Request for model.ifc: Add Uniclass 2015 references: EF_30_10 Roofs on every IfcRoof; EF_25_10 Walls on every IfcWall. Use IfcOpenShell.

First a look at what the model holds.

```python
import ifcopenshell

model = ifcopenshell.open("model.ifc")
print(model.schema)
print("classifications:", [c.Name for c in model.by_type("IfcClassification")])
for ifc_class in ("IfcDoor", "IfcRoof", "IfcStair", "IfcWall", "IfcWindow"):
    print(ifc_class, len(model.by_type(ifc_class)))
```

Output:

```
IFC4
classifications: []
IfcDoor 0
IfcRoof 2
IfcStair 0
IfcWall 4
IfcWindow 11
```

```python
import ifcopenshell
import ifcopenshell.api.classification

model = ifcopenshell.open("model.ifc")

system = ifcopenshell.api.classification.add_classification(model, classification="Uniclass 2015")

codes = {
    "IfcRoof": ("EF_30_10", "Roofs"),
    "IfcWall": ("EF_25_10", "Walls"),
}
for ifc_class, (code, name) in codes.items():
    products = model.by_type(ifc_class)
    ifcopenshell.api.classification.add_reference(
        model, products=products, classification=system, identification=code, name=name
    )
    print(code, len(products))

model.write("model_rev.ifc")
```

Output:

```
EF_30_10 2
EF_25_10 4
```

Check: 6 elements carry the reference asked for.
